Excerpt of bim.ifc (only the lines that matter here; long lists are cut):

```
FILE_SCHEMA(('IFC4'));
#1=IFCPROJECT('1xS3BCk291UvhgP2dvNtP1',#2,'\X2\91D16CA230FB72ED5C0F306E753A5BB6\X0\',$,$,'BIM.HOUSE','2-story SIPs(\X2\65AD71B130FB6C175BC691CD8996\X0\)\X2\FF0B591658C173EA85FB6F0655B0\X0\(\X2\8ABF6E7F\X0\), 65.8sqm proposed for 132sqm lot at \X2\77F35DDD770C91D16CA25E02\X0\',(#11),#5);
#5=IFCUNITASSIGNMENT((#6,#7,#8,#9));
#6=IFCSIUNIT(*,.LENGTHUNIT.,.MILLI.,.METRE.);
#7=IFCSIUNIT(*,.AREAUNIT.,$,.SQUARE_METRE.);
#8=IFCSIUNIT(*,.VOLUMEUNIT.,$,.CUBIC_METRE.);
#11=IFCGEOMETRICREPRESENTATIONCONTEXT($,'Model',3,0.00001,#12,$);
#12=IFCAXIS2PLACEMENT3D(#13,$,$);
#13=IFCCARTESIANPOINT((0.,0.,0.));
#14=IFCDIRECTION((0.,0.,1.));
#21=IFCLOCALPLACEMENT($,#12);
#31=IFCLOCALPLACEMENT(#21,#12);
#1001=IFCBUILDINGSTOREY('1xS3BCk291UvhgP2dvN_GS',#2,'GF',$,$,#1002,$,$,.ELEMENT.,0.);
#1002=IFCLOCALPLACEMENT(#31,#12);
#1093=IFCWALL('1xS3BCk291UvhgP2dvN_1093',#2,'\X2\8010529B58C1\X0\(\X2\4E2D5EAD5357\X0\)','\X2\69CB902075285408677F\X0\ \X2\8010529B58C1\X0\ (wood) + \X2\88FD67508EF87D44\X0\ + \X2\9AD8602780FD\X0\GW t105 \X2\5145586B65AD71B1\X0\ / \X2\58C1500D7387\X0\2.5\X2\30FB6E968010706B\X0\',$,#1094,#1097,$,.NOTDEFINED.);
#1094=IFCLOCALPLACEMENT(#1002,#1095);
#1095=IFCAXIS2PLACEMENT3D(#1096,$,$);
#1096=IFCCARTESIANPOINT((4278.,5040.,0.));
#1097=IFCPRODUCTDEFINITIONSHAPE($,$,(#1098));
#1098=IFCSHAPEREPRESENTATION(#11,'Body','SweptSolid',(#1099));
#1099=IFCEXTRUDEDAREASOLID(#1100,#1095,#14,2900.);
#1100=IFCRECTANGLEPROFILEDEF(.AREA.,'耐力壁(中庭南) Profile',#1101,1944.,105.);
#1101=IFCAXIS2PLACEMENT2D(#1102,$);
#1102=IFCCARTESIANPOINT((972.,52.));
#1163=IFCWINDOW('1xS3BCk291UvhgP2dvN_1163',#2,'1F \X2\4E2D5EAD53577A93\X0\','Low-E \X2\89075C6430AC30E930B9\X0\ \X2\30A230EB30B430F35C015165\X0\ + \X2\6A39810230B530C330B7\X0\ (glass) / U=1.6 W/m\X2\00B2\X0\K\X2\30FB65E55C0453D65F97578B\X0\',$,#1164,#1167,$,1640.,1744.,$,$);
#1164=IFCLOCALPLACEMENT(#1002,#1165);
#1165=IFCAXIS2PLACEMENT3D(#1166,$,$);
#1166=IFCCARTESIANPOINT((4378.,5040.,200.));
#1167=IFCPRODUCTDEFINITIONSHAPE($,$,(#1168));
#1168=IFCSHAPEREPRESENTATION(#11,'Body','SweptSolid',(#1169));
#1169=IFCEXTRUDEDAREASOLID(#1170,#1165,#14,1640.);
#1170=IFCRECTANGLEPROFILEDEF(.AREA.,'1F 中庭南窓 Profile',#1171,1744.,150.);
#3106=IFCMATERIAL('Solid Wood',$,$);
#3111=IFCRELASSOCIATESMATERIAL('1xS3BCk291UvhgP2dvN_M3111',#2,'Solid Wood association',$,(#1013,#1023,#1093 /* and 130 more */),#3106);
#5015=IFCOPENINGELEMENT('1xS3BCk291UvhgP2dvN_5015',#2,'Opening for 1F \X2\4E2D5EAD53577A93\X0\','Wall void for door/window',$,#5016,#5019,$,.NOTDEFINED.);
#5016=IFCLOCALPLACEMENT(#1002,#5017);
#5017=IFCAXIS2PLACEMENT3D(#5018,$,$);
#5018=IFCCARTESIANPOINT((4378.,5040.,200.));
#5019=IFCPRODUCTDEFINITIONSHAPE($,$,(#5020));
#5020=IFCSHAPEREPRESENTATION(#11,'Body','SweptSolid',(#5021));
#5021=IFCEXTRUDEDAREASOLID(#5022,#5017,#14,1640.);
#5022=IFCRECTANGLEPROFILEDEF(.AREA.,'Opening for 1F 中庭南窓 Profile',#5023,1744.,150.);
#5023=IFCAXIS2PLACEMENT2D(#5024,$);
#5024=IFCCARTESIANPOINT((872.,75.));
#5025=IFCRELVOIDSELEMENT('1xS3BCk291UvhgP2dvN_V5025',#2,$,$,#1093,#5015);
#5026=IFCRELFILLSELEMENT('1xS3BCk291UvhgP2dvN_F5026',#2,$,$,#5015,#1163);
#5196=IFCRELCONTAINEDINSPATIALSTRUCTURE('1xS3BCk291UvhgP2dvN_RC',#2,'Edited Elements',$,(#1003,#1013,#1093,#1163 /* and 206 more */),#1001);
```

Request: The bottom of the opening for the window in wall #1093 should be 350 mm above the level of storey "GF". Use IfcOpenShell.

```python
import numpy as np
import ifcopenshell
import ifcopenshell.api.geometry
import ifcopenshell.geom
import ifcopenshell.util.element
import ifcopenshell.util.placement
import ifcopenshell.util.shape
import ifcopenshell.util.unit

model = ifcopenshell.open("bim.ifc")
unit_scale = ifcopenshell.util.unit.calculate_unit_scale(model)

window = model.by_guid("1xS3BCk291UvhgP2dvN_1163")
opening = window.FillsVoids[0].RelatingOpeningElement
storey = ifcopenshell.util.element.get_container(window, ifc_class="IfcBuildingStorey")
level = ifcopenshell.util.placement.get_local_placement(storey.ObjectPlacement)[2, 3]

# The opening's origin need not be at the sill, so measure its lowest point.
shape = ifcopenshell.geom.create_shape(ifcopenshell.geom.settings(), opening)
bottom = ifcopenshell.util.shape.get_shape_bottom_elevation(shape, shape.geometry) / unit_scale
dz = level + 0.35 / unit_scale - bottom

shift = np.array([0.0, 0.0, dz])
# The window is not placed relative to its opening, so move both.
for product in (opening, window):
    matrix = ifcopenshell.util.placement.get_local_placement(product.ObjectPlacement)
    matrix[:3, 3] += shift
    ifcopenshell.api.geometry.edit_object_placement(model, product=product, matrix=matrix, is_si=False)

print(f"moved by {dz * unit_scale:+.3f} m")

model.write("bim_updated.ifc")
```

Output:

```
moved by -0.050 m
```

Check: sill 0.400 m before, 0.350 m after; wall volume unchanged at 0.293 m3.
